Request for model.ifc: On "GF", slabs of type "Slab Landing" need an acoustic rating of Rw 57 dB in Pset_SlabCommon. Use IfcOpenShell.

First a look at what the model holds.

```python
import ifcopenshell
import ifcopenshell.util.element

model = ifcopenshell.open("model.ifc")
print(model.schema)
storey = next(s for s in model.by_type("IfcBuildingStorey") if s.Name == "GF")
slabs = [e for e in ifcopenshell.util.element.get_decomposition(storey) if e.is_a("IfcSlab")]
seen = {}
for e in slabs:
    element_type = ifcopenshell.util.element.get_type(e)
    key = (element_type.Name if element_type != e and element_type else None, ifcopenshell.util.element.get_pset(e, "Pset_SlabCommon", "AcousticRating"))
    seen[key] = seen.get(key, 0) + 1
for (name, value), count in sorted(seen.items(), key=str):
    print(count, "x", name, "|", value)
```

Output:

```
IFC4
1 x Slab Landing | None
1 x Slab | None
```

```python
import ifcopenshell
import ifcopenshell.api.pset
import ifcopenshell.util.element

model = ifcopenshell.open("model.ifc")

storey = next(s for s in model.by_type("IfcBuildingStorey") if s.Name == "GF")
slabs = [e for e in ifcopenshell.util.element.get_decomposition(storey) if e.is_a("IfcSlab")]

count = 0
for e in slabs:
    element_type = ifcopenshell.util.element.get_type(e)
    if element_type in (None, e) or element_type.Name != "Slab Landing":
        continue
    # add_pset returns the element's existing set when there is one.
    pset = ifcopenshell.api.pset.add_pset(model, product=e, name="Pset_SlabCommon")
    ifcopenshell.api.pset.edit_pset(model, pset=pset, properties={"AcousticRating": "Rw 57 dB"})
    count += 1

print(count, "slabs updated")

model.write("model_v2.ifc")
```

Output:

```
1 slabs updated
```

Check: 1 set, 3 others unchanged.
